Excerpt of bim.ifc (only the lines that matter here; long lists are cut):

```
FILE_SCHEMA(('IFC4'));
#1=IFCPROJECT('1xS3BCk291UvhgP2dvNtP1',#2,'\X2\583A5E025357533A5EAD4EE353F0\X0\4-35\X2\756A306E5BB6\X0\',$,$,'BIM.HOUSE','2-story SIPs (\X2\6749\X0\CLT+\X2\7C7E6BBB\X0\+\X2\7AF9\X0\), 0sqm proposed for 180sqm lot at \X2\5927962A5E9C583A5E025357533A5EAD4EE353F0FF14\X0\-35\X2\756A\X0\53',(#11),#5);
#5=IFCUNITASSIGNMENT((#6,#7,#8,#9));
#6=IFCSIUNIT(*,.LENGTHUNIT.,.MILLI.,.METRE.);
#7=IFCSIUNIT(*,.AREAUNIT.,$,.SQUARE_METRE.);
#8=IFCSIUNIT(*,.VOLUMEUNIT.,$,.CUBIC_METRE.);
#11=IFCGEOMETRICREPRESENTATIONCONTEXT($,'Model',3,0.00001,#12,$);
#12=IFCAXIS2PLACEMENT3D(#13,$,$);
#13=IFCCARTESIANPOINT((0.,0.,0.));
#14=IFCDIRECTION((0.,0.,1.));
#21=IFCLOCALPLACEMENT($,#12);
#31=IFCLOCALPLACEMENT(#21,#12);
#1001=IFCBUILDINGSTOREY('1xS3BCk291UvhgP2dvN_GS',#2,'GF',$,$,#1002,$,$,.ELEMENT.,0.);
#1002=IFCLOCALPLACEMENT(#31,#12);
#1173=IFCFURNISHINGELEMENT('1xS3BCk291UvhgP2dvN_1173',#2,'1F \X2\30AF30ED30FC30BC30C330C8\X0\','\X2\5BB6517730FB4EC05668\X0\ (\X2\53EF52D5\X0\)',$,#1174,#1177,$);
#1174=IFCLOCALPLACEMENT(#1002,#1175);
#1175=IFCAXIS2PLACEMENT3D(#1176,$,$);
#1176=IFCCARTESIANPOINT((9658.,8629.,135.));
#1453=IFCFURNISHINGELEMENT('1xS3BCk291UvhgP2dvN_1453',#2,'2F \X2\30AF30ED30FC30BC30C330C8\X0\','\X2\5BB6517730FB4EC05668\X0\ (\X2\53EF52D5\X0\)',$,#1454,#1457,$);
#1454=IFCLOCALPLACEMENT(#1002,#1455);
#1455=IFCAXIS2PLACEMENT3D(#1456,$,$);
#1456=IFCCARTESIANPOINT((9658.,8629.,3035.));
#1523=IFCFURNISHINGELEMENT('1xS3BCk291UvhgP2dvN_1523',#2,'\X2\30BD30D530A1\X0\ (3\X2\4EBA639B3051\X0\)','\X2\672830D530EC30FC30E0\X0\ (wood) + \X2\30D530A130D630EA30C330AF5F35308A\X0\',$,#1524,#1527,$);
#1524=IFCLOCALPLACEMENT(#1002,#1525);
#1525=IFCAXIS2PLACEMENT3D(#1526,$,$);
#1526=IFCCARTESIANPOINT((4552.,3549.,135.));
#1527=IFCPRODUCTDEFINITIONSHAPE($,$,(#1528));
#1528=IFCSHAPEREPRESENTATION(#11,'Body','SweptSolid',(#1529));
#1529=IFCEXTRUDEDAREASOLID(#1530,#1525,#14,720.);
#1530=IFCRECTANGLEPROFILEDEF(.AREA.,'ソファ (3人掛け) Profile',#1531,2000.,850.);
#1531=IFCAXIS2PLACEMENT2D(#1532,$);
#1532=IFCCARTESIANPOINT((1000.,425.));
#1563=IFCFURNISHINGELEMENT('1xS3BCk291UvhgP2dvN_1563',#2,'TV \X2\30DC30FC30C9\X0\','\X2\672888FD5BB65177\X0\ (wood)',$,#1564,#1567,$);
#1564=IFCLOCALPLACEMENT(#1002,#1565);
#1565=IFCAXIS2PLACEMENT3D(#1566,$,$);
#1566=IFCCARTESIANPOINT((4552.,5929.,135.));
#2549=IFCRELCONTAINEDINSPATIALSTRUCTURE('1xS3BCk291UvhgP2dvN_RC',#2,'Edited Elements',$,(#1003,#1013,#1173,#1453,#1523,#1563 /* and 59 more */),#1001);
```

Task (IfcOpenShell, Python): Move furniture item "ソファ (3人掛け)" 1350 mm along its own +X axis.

```python
import ifcopenshell
import ifcopenshell.api.geometry
import ifcopenshell.util.placement
import ifcopenshell.util.unit

model = ifcopenshell.open("bim.ifc")
unit_scale = ifcopenshell.util.unit.calculate_unit_scale(model)

item = model.by_guid("1xS3BCk291UvhgP2dvN_1523")
matrix = ifcopenshell.util.placement.get_local_placement(item.ObjectPlacement)
matrix[:3, 3] += matrix[:3, 0] * 1.35 / unit_scale
ifcopenshell.api.geometry.edit_object_placement(model, product=item, matrix=matrix, is_si=False)

print(ifcopenshell.util.placement.get_local_placement(item.ObjectPlacement).round(3) + 0.0)

model.write("bim_rev.ifc")
```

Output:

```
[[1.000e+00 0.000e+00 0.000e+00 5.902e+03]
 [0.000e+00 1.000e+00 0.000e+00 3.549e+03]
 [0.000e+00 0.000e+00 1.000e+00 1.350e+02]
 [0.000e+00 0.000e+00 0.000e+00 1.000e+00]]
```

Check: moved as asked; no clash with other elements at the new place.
